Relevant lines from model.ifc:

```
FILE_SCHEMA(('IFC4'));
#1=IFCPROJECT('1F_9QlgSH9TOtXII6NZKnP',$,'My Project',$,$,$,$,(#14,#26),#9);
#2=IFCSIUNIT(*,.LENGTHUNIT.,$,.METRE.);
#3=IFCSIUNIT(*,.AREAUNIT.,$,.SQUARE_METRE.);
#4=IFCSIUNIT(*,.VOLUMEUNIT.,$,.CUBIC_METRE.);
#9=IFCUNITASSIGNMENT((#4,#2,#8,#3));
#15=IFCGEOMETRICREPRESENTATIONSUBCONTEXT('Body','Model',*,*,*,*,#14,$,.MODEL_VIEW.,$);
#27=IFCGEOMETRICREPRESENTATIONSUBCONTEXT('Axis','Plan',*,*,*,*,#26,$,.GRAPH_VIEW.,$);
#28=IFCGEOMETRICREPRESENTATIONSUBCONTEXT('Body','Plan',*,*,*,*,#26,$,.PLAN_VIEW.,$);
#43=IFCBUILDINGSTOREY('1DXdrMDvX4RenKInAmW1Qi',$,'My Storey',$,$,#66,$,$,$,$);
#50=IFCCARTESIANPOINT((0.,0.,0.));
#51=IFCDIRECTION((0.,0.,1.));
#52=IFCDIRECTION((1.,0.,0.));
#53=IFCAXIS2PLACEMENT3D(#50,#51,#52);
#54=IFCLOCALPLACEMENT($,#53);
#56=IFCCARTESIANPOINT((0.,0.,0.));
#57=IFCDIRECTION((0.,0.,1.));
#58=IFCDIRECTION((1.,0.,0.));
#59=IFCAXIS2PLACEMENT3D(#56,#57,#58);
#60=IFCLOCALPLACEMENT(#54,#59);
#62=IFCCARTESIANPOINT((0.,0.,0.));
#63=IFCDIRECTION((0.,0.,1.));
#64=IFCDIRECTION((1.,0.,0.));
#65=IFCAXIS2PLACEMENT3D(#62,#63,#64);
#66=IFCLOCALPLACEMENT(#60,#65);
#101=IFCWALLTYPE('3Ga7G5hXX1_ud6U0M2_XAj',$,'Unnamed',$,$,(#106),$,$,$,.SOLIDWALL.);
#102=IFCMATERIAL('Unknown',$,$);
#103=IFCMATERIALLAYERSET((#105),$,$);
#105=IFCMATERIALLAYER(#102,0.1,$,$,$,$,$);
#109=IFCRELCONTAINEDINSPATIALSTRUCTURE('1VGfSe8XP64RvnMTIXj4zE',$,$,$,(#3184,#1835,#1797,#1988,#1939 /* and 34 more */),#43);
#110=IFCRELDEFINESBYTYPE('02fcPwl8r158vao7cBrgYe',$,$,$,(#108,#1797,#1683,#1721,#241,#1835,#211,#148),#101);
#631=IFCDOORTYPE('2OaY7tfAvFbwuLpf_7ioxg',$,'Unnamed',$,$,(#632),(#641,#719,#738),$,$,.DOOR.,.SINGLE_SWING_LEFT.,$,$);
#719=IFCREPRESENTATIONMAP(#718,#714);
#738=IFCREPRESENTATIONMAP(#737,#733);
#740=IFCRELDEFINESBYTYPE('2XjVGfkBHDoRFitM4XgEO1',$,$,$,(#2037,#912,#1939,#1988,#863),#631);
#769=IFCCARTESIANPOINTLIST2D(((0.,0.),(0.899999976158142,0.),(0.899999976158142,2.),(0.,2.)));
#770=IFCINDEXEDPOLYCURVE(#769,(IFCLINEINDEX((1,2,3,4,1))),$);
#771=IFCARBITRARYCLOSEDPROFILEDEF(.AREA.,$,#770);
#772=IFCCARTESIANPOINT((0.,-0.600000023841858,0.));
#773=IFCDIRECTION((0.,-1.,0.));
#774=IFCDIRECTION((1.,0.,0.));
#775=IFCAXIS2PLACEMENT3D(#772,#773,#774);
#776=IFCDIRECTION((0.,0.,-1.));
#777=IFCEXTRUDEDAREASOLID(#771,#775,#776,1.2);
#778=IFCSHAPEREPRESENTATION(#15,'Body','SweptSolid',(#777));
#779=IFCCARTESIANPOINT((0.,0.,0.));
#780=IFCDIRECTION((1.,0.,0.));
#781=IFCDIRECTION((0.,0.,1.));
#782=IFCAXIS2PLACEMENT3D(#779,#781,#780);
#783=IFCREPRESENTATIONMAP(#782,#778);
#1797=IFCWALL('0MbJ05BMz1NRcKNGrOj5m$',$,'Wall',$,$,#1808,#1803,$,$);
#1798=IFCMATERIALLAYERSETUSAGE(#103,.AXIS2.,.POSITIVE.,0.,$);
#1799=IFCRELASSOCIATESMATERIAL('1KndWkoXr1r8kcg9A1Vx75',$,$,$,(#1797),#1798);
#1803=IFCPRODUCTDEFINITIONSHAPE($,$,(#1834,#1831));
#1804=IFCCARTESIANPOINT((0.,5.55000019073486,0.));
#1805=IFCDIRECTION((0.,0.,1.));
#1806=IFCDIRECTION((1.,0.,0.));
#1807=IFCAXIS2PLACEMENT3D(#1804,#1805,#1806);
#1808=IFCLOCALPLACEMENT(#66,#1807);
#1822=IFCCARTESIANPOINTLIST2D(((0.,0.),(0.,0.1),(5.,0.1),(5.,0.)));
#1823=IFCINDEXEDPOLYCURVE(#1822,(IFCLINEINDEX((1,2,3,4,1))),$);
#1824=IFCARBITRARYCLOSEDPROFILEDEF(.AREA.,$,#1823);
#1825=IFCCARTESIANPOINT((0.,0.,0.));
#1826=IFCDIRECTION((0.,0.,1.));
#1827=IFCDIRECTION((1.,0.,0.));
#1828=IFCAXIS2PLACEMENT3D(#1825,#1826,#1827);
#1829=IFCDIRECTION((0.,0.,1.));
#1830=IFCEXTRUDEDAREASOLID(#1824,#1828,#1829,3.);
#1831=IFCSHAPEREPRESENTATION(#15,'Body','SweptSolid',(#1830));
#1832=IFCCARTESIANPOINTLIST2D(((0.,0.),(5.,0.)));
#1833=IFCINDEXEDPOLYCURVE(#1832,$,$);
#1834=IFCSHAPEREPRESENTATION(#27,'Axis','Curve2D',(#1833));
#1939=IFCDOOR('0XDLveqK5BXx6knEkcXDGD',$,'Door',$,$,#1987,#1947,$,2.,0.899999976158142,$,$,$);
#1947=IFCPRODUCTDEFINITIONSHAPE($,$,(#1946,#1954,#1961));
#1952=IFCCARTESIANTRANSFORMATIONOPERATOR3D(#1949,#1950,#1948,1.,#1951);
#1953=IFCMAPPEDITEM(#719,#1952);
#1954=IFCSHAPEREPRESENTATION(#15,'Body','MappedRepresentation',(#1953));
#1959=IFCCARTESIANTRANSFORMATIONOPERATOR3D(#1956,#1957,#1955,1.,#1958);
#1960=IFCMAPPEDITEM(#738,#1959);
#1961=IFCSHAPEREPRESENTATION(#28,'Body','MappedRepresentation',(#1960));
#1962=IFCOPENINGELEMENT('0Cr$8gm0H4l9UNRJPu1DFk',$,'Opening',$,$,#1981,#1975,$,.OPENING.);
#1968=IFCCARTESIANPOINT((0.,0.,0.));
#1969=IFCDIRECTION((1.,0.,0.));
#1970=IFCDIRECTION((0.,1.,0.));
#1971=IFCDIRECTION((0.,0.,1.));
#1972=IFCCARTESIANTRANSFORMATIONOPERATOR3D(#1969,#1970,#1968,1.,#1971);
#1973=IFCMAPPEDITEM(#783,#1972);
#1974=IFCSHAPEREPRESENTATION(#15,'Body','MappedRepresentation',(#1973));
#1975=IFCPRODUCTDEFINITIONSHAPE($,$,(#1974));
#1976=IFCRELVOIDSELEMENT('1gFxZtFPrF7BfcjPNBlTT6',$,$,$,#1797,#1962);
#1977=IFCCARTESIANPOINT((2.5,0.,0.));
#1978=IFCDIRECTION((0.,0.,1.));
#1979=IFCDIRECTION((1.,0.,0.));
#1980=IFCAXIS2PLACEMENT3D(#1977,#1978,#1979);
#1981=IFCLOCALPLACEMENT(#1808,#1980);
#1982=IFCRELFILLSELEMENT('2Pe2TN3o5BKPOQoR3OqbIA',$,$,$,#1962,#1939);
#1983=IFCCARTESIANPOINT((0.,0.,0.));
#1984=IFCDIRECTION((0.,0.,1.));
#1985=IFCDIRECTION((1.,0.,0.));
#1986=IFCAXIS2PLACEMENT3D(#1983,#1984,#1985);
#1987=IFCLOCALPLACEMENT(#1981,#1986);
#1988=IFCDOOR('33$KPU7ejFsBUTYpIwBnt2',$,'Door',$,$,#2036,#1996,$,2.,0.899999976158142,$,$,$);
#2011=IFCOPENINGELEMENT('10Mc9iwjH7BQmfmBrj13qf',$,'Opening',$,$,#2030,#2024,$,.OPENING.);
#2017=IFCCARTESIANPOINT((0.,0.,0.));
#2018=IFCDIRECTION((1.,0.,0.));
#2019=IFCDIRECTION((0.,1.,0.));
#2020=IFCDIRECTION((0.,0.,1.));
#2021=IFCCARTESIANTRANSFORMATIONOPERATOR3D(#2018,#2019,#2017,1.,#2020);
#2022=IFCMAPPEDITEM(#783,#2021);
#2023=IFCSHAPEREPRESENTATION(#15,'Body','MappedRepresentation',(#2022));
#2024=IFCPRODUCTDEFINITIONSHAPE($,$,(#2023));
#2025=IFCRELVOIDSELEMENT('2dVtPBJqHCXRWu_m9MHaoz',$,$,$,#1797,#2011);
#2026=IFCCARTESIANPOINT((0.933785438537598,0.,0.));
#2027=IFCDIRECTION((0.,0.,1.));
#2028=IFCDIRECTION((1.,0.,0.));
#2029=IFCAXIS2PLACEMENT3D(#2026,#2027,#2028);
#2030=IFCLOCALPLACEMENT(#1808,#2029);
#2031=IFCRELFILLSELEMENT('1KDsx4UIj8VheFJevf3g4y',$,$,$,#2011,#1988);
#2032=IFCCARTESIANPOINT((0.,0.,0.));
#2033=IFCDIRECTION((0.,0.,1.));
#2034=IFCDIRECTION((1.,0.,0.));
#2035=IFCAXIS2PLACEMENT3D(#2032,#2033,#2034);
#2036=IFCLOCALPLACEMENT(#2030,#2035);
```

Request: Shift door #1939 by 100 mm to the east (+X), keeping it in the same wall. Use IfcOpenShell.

```python
import ifcopenshell
import ifcopenshell.api.geometry
import ifcopenshell.util.placement
import ifcopenshell.util.unit

model = ifcopenshell.open("model.ifc")
unit_scale = ifcopenshell.util.unit.calculate_unit_scale(model)

door = model.by_id(1939)
opening = door.FillsVoids[0].RelatingOpeningElement
wall = opening.VoidsElements[0].RelatingBuildingElement

wall_matrix = ifcopenshell.util.placement.get_local_placement(wall.ObjectPlacement)
shift = wall_matrix[:3, 0] * 0.1 / unit_scale
before = ifcopenshell.util.placement.get_local_placement(door.ObjectPlacement)[:3, 3].copy()

# The door is placed relative to its opening, so it follows when the opening moves.
matrix = ifcopenshell.util.placement.get_local_placement(opening.ObjectPlacement)
matrix[:3, 3] += shift
ifcopenshell.api.geometry.edit_object_placement(
    model, product=opening, matrix=matrix, is_si=False, should_transform_children=True
)

after = ifcopenshell.util.placement.get_local_placement(door.ObjectPlacement)[:3, 3]
print("door moved by", (after - before).round(3) + 0.0)

model.write("model-out.ifc")
```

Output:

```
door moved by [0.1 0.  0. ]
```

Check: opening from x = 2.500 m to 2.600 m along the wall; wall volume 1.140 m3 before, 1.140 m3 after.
